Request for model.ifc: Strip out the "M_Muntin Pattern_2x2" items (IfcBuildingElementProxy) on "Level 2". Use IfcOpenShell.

First a look at what the model holds.

```python
import ifcopenshell
import ifcopenshell.util.element

model = ifcopenshell.open("model.ifc")
print(model.schema)
storey = next(s for s in model.by_type("IfcBuildingStorey") if s.Name == "Level 2")
proxies = [e for e in ifcopenshell.util.element.get_decomposition(storey) if e.is_a("IfcBuildingElementProxy")]
seen = {}
for e in proxies:
    element_type = ifcopenshell.util.element.get_type(e)
    name = element_type.Name if element_type not in (None, e) else None
    seen[name] = seen.get(name, 0) + 1
for name, count in sorted(seen.items(), key=str):
    print(count, "x", name)
```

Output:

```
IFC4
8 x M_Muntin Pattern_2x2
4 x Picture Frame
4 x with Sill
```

```python
import ifcopenshell
import ifcopenshell.api.root
import ifcopenshell.util.element

model = ifcopenshell.open("model.ifc")

storey = next(s for s in model.by_type("IfcBuildingStorey") if s.Name == "Level 2")
proxies = [e for e in ifcopenshell.util.element.get_decomposition(storey) if e.is_a("IfcBuildingElementProxy")]
targets = [e for e in proxies if (t := ifcopenshell.util.element.get_type(e)) not in (None, e) and t.Name == "M_Muntin Pattern_2x2"]

for e in targets:
    ifcopenshell.api.root.remove_product(model, product=e)
print(len(targets), "removed")

model.write("model_updated.ifc")
```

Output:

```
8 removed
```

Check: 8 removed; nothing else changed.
